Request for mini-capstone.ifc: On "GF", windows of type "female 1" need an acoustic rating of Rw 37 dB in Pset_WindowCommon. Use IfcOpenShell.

First a look at what the model holds.

```python
import ifcopenshell
import ifcopenshell.util.element

model = ifcopenshell.open("mini-capstone.ifc")
print(model.schema)
storey = next(s for s in model.by_type("IfcBuildingStorey") if s.Name == "GF")
windows = [e for e in ifcopenshell.util.element.get_decomposition(storey) if e.is_a("IfcWindow")]
seen = {}
for e in windows:
    element_type = ifcopenshell.util.element.get_type(e)
    key = (element_type.Name if element_type != e and element_type else None, ifcopenshell.util.element.get_pset(e, "Pset_WindowCommon", "AcousticRating"))
    seen[key] = seen.get(key, 0) + 1
for (name, value), count in sorted(seen.items(), key=str):
    print(count, "x", name, "|", value)
```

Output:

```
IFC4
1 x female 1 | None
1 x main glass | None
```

```python
import ifcopenshell
import ifcopenshell.api.pset
import ifcopenshell.util.element

model = ifcopenshell.open("mini-capstone.ifc")

storey = next(s for s in model.by_type("IfcBuildingStorey") if s.Name == "GF")
windows = [e for e in ifcopenshell.util.element.get_decomposition(storey) if e.is_a("IfcWindow")]

count = 0
for e in windows:
    element_type = ifcopenshell.util.element.get_type(e)
    if element_type in (None, e) or element_type.Name != "female 1":
        continue
    # add_pset returns the element's existing set when there is one.
    pset = ifcopenshell.api.pset.add_pset(model, product=e, name="Pset_WindowCommon")
    ifcopenshell.api.pset.edit_pset(model, pset=pset, properties={"AcousticRating": "Rw 37 dB"})
    count += 1

print(count, "windows updated")

model.write("mini-capstone_updated.ifc")
```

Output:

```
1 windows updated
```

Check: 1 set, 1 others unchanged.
